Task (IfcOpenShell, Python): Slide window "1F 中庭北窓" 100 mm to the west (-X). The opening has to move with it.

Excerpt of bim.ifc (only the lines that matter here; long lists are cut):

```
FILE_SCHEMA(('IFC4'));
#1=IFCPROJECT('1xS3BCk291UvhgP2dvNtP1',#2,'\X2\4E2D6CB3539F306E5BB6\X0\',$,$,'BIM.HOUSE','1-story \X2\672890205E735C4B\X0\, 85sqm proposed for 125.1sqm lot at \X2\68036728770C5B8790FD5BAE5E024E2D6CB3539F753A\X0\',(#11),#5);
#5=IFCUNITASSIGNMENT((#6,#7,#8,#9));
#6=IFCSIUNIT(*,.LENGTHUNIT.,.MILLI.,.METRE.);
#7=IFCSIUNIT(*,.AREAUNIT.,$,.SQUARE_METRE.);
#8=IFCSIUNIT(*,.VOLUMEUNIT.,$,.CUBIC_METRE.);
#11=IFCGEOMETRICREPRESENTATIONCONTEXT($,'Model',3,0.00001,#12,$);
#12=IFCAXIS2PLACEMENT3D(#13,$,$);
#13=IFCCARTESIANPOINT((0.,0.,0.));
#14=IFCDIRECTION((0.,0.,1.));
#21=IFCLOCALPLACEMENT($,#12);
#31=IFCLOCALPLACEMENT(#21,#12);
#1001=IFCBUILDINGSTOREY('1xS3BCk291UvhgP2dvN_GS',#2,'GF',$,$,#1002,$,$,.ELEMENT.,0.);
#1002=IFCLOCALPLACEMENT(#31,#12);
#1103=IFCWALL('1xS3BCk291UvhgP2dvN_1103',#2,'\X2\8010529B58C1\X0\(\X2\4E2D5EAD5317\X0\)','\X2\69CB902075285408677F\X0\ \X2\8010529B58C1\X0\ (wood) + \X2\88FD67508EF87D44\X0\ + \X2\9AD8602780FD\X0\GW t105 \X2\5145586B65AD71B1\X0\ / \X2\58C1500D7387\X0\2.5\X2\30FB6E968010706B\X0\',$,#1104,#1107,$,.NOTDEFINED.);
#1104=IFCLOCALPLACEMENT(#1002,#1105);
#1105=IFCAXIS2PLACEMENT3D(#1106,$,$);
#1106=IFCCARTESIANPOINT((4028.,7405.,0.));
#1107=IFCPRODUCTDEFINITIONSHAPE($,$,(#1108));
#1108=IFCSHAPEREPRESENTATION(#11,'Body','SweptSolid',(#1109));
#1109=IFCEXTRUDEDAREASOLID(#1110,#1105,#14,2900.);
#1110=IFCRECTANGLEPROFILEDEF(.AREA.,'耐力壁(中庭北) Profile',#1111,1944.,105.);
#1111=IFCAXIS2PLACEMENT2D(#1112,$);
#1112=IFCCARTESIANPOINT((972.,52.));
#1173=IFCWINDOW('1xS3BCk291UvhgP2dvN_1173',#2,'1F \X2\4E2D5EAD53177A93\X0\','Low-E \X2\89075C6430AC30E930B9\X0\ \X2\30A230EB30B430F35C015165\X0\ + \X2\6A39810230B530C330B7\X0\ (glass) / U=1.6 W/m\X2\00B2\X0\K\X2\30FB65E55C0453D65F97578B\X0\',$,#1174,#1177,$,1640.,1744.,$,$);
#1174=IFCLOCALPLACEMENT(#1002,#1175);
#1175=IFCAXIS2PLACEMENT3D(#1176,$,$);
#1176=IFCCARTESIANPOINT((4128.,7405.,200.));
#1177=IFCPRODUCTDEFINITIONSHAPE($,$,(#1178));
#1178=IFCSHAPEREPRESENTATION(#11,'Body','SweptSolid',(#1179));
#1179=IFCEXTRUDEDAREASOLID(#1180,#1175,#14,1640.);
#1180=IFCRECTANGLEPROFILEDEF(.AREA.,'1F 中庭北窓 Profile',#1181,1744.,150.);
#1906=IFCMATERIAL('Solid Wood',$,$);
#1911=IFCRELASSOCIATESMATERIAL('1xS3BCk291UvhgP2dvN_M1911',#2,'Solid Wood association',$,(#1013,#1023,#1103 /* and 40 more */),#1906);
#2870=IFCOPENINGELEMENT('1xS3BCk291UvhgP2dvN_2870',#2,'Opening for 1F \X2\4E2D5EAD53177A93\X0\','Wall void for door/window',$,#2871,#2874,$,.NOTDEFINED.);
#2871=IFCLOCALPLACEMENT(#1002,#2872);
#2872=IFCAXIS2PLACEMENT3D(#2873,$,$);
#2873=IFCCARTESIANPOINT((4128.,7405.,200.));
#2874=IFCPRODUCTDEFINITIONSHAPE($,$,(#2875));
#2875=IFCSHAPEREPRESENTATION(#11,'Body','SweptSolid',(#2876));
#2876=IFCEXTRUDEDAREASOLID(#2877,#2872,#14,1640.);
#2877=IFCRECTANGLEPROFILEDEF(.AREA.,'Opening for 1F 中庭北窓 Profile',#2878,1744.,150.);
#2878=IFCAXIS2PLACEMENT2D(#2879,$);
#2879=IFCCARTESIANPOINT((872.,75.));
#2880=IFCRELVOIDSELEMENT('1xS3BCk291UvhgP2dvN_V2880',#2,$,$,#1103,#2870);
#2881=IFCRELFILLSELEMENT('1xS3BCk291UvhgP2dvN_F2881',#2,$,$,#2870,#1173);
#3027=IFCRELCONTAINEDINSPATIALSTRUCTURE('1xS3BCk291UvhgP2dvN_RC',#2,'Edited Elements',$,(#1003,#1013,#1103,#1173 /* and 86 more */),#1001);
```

```python
import ifcopenshell
import ifcopenshell.api.geometry
import ifcopenshell.util.placement

model = ifcopenshell.open("bim.ifc")

window = model.by_guid("1xS3BCk291UvhgP2dvN_1173")
opening = window.FillsVoids[0].RelatingOpeningElement
wall = opening.VoidsElements[0].RelatingBuildingElement

wall_matrix = ifcopenshell.util.placement.get_local_placement(wall.ObjectPlacement)
shift = wall_matrix[:3, 0] * -100.0
before = ifcopenshell.util.placement.get_local_placement(window.ObjectPlacement)[:3, 3].copy()

# The window is not placed relative to its opening, so move both.
for product in (opening, window):
    matrix = ifcopenshell.util.placement.get_local_placement(product.ObjectPlacement)
    matrix[:3, 3] += shift
    ifcopenshell.api.geometry.edit_object_placement(model, product=product, matrix=matrix, is_si=False)

after = ifcopenshell.util.placement.get_local_placement(window.ObjectPlacement)[:3, 3]
print("window moved by", (after - before).round(3) + 0.0)

model.write("bim_edited.ifc")
```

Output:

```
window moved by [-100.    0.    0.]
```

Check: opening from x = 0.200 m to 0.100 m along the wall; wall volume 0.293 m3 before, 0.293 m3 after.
